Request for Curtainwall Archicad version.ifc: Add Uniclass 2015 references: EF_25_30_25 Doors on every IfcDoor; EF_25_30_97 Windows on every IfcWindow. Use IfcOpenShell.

First a look at what the model holds.

```python
import ifcopenshell

model = ifcopenshell.open("Curtainwall Archicad version.ifc")
print(model.schema)
print("classifications:", [c.Name for c in model.by_type("IfcClassification")])
for ifc_class in ("IfcDoor", "IfcRoof", "IfcStair", "IfcWall", "IfcWindow"):
    print(ifc_class, len(model.by_type(ifc_class)))
```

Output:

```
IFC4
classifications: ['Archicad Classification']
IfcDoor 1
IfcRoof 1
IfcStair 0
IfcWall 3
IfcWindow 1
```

```python
import ifcopenshell
import ifcopenshell.api.classification

model = ifcopenshell.open("Curtainwall Archicad version.ifc")

system = ifcopenshell.api.classification.add_classification(model, classification="Uniclass 2015")

codes = {
    "IfcDoor": ("EF_25_30_25", "Doors"),
    "IfcWindow": ("EF_25_30_97", "Windows"),
}
for ifc_class, (code, name) in codes.items():
    products = model.by_type(ifc_class)
    ifcopenshell.api.classification.add_reference(
        model, products=products, classification=system, identification=code, name=name
    )
    print(code, len(products))

model.write("Curtainwall Archicad version_edited.ifc")
```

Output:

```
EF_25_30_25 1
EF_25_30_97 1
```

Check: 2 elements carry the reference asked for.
